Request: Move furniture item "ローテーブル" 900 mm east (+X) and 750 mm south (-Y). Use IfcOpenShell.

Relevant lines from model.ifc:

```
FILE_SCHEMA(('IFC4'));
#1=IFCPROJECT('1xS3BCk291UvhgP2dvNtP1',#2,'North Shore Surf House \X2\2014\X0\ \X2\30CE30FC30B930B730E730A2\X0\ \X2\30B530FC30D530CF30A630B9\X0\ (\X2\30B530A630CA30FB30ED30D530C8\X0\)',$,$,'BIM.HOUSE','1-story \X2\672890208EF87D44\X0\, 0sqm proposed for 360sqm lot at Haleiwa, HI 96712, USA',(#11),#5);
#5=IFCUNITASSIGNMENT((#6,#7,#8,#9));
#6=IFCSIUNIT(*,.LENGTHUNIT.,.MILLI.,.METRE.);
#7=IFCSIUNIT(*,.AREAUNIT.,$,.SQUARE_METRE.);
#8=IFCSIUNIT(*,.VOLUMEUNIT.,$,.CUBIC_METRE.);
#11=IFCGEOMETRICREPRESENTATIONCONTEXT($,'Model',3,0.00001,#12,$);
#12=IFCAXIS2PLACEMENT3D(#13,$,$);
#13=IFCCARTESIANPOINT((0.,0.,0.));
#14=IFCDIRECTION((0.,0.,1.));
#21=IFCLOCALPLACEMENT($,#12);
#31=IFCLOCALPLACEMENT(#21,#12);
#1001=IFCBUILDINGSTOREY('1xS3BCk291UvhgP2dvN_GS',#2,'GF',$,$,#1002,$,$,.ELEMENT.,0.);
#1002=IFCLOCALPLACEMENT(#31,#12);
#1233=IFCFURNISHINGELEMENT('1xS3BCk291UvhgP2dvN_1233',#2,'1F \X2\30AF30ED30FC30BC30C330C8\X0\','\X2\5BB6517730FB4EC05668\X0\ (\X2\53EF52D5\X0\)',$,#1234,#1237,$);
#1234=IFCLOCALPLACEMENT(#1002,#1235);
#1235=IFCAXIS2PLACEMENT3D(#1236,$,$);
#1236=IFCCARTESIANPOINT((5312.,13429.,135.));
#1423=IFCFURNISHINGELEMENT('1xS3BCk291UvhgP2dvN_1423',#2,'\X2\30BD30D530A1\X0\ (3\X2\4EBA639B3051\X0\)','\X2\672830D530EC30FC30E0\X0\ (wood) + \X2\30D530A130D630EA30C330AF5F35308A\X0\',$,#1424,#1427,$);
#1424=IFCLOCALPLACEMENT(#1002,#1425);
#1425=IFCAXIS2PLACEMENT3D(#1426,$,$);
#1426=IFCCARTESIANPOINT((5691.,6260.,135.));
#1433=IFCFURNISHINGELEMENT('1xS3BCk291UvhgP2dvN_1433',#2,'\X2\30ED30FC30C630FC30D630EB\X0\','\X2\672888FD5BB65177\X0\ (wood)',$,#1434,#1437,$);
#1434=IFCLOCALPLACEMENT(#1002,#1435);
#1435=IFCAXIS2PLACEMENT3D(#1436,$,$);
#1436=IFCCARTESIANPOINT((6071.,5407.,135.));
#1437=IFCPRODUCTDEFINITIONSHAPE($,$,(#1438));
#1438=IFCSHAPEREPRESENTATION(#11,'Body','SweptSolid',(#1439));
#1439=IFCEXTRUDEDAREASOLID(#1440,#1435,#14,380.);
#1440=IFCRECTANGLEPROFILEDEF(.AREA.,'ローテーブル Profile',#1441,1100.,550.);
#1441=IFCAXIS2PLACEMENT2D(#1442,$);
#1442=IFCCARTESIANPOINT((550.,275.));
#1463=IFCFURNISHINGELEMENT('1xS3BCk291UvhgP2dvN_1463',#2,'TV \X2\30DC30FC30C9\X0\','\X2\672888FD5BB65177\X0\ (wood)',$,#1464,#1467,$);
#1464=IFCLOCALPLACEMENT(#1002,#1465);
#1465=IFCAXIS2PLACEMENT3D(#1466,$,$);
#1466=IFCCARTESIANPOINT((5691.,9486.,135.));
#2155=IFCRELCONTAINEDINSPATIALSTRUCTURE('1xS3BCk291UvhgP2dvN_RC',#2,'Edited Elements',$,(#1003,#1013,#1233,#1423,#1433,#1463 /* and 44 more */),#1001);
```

```python
import ifcopenshell
import ifcopenshell.api.geometry
import ifcopenshell.util.placement

model = ifcopenshell.open("model.ifc")

item = model.by_id(1433)
matrix = ifcopenshell.util.placement.get_local_placement(item.ObjectPlacement)
matrix[0, 3] += 900.0
matrix[1, 3] -= 750.0
ifcopenshell.api.geometry.edit_object_placement(model, product=item, matrix=matrix, is_si=False)

print(ifcopenshell.util.placement.get_local_placement(item.ObjectPlacement).round(3) + 0.0)

model.write("model_edited.ifc")
```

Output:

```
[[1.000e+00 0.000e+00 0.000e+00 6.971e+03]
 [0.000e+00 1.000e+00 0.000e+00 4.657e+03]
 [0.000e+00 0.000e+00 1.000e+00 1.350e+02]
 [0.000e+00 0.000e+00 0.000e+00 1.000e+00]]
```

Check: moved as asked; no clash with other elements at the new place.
